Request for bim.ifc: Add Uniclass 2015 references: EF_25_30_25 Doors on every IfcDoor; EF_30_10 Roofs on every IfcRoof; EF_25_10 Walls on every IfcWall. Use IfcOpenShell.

First a look at what the model holds.

```python
import ifcopenshell

model = ifcopenshell.open("bim.ifc")
print(model.schema)
print("classifications:", [c.Name for c in model.by_type("IfcClassification")])
for ifc_class in ("IfcDoor", "IfcRoof", "IfcStair", "IfcWall", "IfcWindow"):
    print(ifc_class, len(model.by_type(ifc_class)))
```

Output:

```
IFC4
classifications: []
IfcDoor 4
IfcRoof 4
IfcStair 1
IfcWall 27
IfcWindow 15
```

```python
import ifcopenshell
import ifcopenshell.api.classification

model = ifcopenshell.open("bim.ifc")

system = ifcopenshell.api.classification.add_classification(model, classification="Uniclass 2015")

codes = {
    "IfcDoor": ("EF_25_30_25", "Doors"),
    "IfcRoof": ("EF_30_10", "Roofs"),
    "IfcWall": ("EF_25_10", "Walls"),
}
for ifc_class, (code, name) in codes.items():
    products = model.by_type(ifc_class)
    ifcopenshell.api.classification.add_reference(
        model, products=products, classification=system, identification=code, name=name
    )
    print(code, len(products))

model.write("bim-out.ifc")
```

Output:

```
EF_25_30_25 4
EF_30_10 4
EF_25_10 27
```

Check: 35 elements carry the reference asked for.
